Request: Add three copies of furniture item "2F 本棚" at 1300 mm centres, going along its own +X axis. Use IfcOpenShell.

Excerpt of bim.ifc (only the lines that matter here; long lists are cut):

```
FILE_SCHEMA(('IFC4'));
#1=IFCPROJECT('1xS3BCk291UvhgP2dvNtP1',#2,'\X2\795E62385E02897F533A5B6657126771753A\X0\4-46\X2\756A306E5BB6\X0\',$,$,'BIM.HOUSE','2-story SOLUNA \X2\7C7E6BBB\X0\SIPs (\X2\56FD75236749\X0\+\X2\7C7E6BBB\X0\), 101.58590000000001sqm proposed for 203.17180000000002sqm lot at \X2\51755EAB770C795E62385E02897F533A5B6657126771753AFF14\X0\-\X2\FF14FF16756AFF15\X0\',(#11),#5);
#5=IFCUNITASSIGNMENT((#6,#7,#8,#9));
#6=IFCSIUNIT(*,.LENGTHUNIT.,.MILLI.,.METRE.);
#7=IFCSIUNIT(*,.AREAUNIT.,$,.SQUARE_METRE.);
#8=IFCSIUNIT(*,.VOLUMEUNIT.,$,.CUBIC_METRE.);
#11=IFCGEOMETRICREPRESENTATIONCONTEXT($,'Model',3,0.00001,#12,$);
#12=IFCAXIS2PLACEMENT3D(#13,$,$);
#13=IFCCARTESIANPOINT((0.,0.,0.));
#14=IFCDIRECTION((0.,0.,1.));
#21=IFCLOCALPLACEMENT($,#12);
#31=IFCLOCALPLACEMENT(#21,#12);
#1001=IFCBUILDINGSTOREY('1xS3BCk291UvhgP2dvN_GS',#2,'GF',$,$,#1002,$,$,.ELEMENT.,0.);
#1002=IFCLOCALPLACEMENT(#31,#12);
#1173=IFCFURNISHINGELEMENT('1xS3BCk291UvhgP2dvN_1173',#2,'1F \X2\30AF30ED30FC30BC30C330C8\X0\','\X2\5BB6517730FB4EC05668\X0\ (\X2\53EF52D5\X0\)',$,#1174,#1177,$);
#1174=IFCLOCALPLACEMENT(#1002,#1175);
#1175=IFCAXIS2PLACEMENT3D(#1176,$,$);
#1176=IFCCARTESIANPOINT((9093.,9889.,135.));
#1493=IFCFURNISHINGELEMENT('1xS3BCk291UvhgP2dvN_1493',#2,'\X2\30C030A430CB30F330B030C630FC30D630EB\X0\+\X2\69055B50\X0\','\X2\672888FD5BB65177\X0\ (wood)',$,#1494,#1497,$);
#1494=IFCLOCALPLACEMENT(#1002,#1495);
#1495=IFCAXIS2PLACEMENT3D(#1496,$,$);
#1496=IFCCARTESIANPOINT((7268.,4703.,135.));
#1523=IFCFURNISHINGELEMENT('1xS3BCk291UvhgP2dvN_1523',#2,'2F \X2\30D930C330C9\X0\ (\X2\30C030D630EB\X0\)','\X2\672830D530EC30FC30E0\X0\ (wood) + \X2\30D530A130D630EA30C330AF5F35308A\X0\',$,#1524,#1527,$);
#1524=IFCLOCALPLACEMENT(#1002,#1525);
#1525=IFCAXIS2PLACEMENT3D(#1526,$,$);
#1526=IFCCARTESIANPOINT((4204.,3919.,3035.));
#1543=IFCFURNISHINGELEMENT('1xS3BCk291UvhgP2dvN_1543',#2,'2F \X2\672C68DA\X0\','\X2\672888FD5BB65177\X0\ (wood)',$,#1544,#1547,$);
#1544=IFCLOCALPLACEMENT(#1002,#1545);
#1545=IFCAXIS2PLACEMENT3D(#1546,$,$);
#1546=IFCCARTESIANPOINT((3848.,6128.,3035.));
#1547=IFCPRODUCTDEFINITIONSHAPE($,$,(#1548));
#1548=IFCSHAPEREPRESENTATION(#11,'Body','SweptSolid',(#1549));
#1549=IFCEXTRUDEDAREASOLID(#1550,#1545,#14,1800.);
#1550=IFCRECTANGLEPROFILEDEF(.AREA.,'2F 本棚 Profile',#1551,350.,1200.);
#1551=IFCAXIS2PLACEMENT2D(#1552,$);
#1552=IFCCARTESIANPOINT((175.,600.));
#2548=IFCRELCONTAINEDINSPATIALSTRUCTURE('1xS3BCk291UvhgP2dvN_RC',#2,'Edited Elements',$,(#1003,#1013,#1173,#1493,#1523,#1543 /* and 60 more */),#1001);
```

```python
import ifcopenshell
import ifcopenshell.api.geometry
import ifcopenshell.api.root
import ifcopenshell.util.element
import ifcopenshell.util.placement
import ifcopenshell.util.unit

model = ifcopenshell.open("bim.ifc")
unit_scale = ifcopenshell.util.unit.calculate_unit_scale(model)


def reuse_history(source, copy):
    """copy_class also copies each property set's owner history, people and application; keep the originals."""
    for rel in copy.IsDefinedBy:
        if rel.is_a("IfcRelDefinesByProperties") and (history := rel.RelatingPropertyDefinition.OwnerHistory):
            rel.RelatingPropertyDefinition.OwnerHistory = source.OwnerHistory
            ifcopenshell.util.element.remove_deep2(model, history)


source = model.by_guid("1xS3BCk291UvhgP2dvN_1543")
base = ifcopenshell.util.placement.get_local_placement(source.ObjectPlacement)
step = base[:3, 0] * 1.3 / unit_scale

for i in range(1, 4):
    copy = ifcopenshell.api.root.copy_class(model, product=source)
    copy.Representation = ifcopenshell.util.element.copy_deep(
        model, source.Representation, exclude=["IfcGeometricRepresentationContext", "IfcRepresentationMap"]
    )
    reuse_history(source, copy)
    matrix = base.copy()
    matrix[:3, 3] += i * step
    print("added at", matrix[:3, 3].round(3) + 0.0)
    ifcopenshell.api.geometry.edit_object_placement(model, product=copy, matrix=matrix, is_si=False)

model.write("bim_updated.ifc")
```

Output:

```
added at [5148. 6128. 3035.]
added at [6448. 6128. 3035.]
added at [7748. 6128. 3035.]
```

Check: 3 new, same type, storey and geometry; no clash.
